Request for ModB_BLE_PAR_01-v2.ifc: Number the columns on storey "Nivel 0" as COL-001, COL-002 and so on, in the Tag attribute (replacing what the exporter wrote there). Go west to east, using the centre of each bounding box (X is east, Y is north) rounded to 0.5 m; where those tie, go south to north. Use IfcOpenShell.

First a look at what the model holds.

```python
import ifcopenshell
import ifcopenshell.util.element
import ifcopenshell.util.placement

model = ifcopenshell.open("ModB_BLE_PAR_01-v2.ifc")
print(model.schema)
storey = next(s for s in model.by_type("IfcBuildingStorey") if s.Name == "Nivel 0")
columns = [e for e in ifcopenshell.util.element.get_decomposition(storey) if e.is_a("IfcColumn")]
for e in sorted(columns, key=lambda e: e.id()):
    origin = ifcopenshell.util.placement.get_local_placement(e.ObjectPlacement)[:3, 3]
    print(e.id(), e.Tag, e.Name, origin.round(2) + 0.0, sep=" | ")
```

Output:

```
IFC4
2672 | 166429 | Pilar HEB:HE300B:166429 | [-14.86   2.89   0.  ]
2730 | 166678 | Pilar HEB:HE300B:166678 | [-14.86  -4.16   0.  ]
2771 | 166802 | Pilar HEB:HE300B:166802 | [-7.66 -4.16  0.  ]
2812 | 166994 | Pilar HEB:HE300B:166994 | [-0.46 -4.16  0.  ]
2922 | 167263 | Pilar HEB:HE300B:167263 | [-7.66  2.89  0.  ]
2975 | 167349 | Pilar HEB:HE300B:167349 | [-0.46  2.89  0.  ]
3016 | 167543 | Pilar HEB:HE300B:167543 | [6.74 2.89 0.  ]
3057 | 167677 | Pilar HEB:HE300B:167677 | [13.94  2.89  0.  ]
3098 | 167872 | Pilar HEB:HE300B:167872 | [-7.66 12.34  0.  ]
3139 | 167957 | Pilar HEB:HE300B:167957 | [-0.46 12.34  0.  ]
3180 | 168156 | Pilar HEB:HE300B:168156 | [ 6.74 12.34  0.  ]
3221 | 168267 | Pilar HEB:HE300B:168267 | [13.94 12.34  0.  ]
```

```python
import ifcopenshell
import ifcopenshell.geom
import ifcopenshell.util.element
import ifcopenshell.util.shape

model = ifcopenshell.open("ModB_BLE_PAR_01-v2.ifc")
settings = ifcopenshell.geom.settings()
settings.set("use-world-coords", True)


def centre(element):
    shape = ifcopenshell.geom.create_shape(settings, element)
    return ifcopenshell.util.shape.get_bbox_centroid(shape.geometry)


storey = next(s for s in model.by_type("IfcBuildingStorey") if s.Name == "Nivel 0")
columns = [e for e in ifcopenshell.util.element.get_decomposition(storey) if e.is_a("IfcColumn")]

# Insertion points can sit at a corner or the storey origin, so sort by the geometry (in metres).
centres = {e: centre(e) for e in columns}
columns.sort(key=lambda e: (round(centres[e][0] / 0.5), centres[e][1]))

for i, e in enumerate(columns, start=1):
    number = f"COL-0{i:02d}"
    e.Tag = number
    print(e.id(), number)

model.write("ModB_BLE_PAR_01-v2_updated.ifc")
```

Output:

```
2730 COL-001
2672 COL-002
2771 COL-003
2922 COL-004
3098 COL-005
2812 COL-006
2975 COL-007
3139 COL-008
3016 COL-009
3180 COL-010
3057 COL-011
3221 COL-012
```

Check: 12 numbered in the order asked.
